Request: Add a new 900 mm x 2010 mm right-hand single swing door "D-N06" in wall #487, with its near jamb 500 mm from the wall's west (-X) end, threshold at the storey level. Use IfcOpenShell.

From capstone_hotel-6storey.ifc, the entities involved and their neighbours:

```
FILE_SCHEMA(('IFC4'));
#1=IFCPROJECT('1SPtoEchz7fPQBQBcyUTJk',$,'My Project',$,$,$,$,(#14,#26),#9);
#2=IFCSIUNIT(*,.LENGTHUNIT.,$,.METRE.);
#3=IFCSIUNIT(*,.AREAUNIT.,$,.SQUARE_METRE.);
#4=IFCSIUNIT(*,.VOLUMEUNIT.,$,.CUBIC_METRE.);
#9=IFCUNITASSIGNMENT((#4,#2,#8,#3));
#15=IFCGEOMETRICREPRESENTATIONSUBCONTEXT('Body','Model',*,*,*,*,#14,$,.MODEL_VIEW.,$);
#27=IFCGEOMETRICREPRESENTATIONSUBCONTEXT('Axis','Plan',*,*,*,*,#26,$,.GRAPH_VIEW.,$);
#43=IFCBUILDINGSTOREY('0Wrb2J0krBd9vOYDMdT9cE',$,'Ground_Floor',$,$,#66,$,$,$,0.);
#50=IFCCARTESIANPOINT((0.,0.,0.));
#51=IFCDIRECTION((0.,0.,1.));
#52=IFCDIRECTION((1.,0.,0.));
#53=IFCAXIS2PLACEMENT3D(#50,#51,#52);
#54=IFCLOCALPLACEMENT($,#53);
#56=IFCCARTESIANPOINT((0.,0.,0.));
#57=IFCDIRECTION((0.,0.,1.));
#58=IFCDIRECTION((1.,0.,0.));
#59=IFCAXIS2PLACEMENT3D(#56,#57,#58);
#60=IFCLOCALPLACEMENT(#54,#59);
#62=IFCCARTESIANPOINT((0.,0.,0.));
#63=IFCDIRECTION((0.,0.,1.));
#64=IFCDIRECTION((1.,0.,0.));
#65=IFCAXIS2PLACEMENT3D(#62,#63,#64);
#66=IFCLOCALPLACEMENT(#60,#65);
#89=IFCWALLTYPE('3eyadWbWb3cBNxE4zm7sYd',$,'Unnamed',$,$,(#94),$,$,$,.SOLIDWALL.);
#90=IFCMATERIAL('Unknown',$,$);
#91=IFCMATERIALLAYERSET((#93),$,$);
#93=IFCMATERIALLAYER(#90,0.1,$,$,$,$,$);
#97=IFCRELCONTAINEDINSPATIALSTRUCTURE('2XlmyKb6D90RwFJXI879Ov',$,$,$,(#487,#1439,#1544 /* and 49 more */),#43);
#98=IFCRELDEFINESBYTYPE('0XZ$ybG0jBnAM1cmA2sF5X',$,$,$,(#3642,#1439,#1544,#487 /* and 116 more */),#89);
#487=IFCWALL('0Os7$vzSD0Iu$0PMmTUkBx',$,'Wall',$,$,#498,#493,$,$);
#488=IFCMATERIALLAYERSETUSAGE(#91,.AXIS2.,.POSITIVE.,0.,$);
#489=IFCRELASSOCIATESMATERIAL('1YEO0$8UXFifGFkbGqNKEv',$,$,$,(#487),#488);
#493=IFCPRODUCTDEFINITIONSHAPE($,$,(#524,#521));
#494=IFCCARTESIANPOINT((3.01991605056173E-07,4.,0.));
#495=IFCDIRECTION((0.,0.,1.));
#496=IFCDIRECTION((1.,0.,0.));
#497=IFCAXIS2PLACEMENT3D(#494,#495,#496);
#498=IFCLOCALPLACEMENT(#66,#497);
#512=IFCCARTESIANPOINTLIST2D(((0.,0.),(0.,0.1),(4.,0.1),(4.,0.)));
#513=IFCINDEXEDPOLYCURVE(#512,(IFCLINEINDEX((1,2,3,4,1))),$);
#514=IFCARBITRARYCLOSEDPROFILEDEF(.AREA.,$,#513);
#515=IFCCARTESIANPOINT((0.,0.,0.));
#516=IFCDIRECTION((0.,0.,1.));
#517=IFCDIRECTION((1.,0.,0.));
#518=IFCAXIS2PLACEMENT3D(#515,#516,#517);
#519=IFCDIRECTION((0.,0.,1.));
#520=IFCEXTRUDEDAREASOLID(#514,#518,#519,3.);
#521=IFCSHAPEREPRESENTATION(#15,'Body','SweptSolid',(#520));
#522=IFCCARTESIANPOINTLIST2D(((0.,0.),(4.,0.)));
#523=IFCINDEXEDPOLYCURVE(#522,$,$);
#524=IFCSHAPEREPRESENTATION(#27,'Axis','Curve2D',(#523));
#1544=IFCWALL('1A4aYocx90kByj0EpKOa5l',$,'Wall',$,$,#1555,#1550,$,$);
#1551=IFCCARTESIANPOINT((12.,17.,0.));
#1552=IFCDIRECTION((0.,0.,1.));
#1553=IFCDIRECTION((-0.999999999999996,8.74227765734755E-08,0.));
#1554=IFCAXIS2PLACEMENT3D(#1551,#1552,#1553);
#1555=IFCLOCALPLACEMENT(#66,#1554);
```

```python
import numpy as np
import ifcopenshell
import ifcopenshell.api.feature
import ifcopenshell.api.geometry
import ifcopenshell.api.root
import ifcopenshell.api.spatial
import ifcopenshell.geom
import ifcopenshell.util.element
import ifcopenshell.util.placement
import ifcopenshell.util.representation
import ifcopenshell.util.shape
import ifcopenshell.util.unit

model = ifcopenshell.open("capstone_hotel-6storey.ifc")
unit_scale = ifcopenshell.util.unit.calculate_unit_scale(model)
settings = ifcopenshell.geom.settings()


def volume(element):
    """Net volume in cubic metres, openings subtracted."""
    shape = ifcopenshell.geom.create_shape(settings, element)
    return ifcopenshell.util.shape.get_volume(shape.geometry)


wall = model.by_guid("0Os7$vzSD0Iu$0PMmTUkBx")
storey = ifcopenshell.util.element.get_container(wall, ifc_class="IfcBuildingStorey")
context = ifcopenshell.util.representation.get_context(model, "Model", "Body", "MODEL_VIEW")
before = volume(wall)

width, height, from_end, sill = 0.9, 2.01, 0.5, 0.0  # metres

# The wall runs along its own X axis, and the end named is its -X end.
wall_shape = ifcopenshell.geom.create_shape(settings, wall)
x, y, z = ifcopenshell.util.shape.get_vertices(wall_shape.geometry).T
start = x.min() + from_end
face, thickness = float(y.min()), float(y.max() - y.min())
wall_matrix = ifcopenshell.util.placement.get_local_placement(wall.ObjectPlacement)
level = ifcopenshell.util.placement.get_local_placement(storey.ObjectPlacement)[2, 3]


def in_wall(x, y):
    """Placement at x, y metres in the wall's axes, at sill height."""
    matrix = wall_matrix.copy()
    matrix[:, 3] = wall_matrix @ np.array([x / unit_scale, y / unit_scale, 0.0, 1.0])
    matrix[2, 3] = level + sill / unit_scale
    return matrix


# Opening: a box that overshoots both wall faces by 50 mm.
opening = ifcopenshell.api.root.create_entity(model, ifc_class="IfcOpeningElement", predefined_type="OPENING")
box = ifcopenshell.api.geometry.add_wall_representation(
    model, context=context, length=width, height=height, thickness=thickness + 0.1
)
ifcopenshell.api.geometry.assign_representation(model, product=opening, representation=box)
ifcopenshell.api.geometry.edit_object_placement(model, product=opening, matrix=in_wall(start, face - 0.05), is_si=False)
ifcopenshell.api.feature.add_feature(model, feature=opening, element=wall)

door = ifcopenshell.api.root.create_entity(model, ifc_class="IfcDoor", name="D-N06", predefined_type="DOOR")
door.OverallWidth, door.OverallHeight = width / unit_scale, height / unit_scale
door.OperationType = "SINGLE_SWING_RIGHT"
body = ifcopenshell.api.geometry.add_door_representation(
    model,
    context=context,
    overall_width=door.OverallWidth,
    overall_height=door.OverallHeight,
    operation_type="SINGLE_SWING_RIGHT",
    lining_properties={"LiningDepth": thickness / unit_scale, "ThresholdDepth": thickness / unit_scale},
)
ifcopenshell.api.geometry.assign_representation(model, product=door, representation=body)
ifcopenshell.api.spatial.assign_container(model, products=[door], relating_structure=storey)
ifcopenshell.api.feature.add_filling(model, opening=opening, element=door)

# The lining spans the wall, so the door starts at the wall face.
ifcopenshell.api.geometry.edit_object_placement(model, product=door, matrix=in_wall(start, face), is_si=False)

after = volume(wall)

print(f"wall volume {before:.3f} -> {after:.3f} m3")

model.write("capstone_hotel-6storey_v2.ifc")
```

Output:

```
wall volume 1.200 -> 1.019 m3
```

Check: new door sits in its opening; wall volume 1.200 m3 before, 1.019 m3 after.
